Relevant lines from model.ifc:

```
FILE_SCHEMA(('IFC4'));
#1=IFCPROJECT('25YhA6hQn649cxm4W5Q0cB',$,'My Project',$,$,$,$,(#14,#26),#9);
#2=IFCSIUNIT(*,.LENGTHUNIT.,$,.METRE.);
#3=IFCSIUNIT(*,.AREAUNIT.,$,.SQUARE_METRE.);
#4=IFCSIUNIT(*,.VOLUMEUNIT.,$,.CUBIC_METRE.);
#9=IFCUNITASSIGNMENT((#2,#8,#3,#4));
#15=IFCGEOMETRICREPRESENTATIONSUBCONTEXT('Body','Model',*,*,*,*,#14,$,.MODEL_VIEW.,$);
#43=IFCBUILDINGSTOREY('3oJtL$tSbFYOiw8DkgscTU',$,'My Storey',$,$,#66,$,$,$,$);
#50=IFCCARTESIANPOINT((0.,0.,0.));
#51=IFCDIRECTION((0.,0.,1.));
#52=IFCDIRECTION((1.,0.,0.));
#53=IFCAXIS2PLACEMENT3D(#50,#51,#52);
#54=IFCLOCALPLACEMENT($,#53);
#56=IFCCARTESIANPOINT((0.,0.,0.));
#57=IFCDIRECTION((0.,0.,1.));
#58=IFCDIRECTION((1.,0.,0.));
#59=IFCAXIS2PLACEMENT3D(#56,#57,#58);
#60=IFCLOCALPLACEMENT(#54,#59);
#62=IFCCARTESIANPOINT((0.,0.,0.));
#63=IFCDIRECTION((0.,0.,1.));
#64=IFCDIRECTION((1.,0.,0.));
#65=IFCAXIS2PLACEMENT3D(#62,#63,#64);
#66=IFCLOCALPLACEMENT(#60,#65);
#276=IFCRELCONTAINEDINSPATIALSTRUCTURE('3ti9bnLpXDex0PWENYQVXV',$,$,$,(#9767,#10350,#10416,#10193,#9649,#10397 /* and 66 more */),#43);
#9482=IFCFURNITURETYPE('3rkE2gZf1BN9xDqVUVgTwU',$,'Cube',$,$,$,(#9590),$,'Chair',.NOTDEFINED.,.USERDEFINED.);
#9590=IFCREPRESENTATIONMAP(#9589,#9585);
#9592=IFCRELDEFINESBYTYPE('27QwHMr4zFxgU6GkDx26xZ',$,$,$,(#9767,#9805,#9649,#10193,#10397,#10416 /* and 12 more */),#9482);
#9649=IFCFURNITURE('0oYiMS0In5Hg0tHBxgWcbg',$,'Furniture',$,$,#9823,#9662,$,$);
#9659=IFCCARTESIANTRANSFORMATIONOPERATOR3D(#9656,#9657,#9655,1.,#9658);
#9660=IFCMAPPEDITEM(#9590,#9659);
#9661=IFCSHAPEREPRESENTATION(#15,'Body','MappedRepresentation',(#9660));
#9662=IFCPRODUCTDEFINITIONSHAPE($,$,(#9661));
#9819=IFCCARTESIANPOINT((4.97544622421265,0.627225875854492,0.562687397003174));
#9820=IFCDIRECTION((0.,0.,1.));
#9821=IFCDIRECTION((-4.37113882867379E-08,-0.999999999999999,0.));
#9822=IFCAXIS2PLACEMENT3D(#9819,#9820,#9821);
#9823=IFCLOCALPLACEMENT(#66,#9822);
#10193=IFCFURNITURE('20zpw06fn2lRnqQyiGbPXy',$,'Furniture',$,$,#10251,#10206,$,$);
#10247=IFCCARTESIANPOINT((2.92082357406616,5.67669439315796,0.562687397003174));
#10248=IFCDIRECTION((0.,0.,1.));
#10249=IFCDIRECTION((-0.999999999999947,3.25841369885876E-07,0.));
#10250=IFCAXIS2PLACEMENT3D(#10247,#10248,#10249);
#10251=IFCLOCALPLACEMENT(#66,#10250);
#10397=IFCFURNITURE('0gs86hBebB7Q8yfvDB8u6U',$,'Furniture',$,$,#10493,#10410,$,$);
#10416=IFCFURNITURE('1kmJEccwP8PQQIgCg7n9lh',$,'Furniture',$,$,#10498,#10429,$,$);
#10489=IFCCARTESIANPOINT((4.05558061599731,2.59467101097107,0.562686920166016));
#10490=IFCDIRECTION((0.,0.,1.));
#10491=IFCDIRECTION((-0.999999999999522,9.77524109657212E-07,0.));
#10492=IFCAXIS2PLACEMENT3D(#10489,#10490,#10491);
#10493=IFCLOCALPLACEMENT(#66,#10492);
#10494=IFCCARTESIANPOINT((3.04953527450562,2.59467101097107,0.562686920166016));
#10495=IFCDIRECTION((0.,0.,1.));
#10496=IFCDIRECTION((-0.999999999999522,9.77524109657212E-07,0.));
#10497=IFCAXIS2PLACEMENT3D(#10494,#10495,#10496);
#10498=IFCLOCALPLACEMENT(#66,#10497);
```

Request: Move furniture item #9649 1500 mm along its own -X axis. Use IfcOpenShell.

```python
import ifcopenshell
import ifcopenshell.api.geometry
import ifcopenshell.util.placement
import ifcopenshell.util.unit

model = ifcopenshell.open("model.ifc")
unit_scale = ifcopenshell.util.unit.calculate_unit_scale(model)

item = model.by_guid("0oYiMS0In5Hg0tHBxgWcbg")
matrix = ifcopenshell.util.placement.get_local_placement(item.ObjectPlacement)
matrix[:3, 3] -= matrix[:3, 0] * 1.5 / unit_scale
ifcopenshell.api.geometry.edit_object_placement(model, product=item, matrix=matrix, is_si=False)

print(ifcopenshell.util.placement.get_local_placement(item.ObjectPlacement).round(3) + 0.0)

model.write("model_rev.ifc")
```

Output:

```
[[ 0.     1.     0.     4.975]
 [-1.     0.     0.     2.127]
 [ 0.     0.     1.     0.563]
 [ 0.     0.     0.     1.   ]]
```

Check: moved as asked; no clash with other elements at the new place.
